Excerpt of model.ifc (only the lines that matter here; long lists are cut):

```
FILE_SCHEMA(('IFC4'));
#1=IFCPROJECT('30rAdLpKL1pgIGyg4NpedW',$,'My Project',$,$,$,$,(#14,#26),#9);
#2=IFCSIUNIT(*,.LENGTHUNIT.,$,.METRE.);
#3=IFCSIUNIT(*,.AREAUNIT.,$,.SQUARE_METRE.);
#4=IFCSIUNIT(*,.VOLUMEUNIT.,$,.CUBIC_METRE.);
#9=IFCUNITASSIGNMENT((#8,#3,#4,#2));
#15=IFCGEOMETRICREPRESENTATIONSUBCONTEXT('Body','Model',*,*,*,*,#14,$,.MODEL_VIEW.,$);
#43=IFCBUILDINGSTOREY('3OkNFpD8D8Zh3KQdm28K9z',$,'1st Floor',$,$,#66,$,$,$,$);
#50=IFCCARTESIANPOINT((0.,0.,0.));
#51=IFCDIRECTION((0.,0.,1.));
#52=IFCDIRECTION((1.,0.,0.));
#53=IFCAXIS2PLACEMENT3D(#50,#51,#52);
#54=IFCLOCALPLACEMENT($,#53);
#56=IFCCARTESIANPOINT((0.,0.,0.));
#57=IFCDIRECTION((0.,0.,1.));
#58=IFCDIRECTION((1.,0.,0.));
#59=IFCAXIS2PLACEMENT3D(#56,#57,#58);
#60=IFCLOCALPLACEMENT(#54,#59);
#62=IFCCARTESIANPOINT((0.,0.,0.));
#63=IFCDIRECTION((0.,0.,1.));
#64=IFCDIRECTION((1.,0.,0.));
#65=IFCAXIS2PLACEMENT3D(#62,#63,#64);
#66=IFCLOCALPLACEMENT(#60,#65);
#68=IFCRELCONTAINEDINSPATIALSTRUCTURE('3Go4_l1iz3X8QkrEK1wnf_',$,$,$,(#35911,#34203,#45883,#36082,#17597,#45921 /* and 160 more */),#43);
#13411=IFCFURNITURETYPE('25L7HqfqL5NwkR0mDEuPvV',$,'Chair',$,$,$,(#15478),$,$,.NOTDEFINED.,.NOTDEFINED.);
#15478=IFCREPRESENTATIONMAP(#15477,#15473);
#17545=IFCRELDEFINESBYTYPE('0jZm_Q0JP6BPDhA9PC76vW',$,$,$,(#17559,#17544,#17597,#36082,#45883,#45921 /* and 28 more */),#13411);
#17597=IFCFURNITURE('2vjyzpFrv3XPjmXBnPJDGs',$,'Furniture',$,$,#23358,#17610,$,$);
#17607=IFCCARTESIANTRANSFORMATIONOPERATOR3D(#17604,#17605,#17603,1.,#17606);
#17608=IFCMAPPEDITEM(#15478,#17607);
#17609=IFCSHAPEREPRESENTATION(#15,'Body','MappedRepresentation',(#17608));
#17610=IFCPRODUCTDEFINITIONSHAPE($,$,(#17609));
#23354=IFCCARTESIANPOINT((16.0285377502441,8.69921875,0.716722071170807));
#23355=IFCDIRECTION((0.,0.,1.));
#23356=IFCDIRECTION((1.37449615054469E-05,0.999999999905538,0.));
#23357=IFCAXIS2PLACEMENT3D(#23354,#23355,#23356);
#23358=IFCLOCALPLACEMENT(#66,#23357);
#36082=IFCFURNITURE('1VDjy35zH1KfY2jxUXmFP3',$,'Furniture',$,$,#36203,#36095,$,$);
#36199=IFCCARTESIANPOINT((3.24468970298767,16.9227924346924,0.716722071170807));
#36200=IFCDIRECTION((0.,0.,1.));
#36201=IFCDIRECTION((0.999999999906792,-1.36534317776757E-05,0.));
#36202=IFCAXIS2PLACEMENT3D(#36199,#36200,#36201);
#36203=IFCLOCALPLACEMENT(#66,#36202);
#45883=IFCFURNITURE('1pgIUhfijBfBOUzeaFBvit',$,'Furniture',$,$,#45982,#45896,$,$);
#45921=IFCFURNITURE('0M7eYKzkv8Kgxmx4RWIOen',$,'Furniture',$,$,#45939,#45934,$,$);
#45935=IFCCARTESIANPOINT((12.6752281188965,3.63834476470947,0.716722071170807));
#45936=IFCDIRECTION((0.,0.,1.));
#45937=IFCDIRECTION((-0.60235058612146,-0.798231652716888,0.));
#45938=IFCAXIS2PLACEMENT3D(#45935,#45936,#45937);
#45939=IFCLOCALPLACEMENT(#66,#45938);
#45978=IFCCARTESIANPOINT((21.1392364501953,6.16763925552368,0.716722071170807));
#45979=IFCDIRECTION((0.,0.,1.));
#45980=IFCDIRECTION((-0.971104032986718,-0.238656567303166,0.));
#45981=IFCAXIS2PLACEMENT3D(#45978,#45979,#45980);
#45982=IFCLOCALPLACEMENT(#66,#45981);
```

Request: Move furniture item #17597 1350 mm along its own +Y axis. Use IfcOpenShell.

```python
import ifcopenshell
import ifcopenshell.api.geometry
import ifcopenshell.util.placement
import ifcopenshell.util.unit

model = ifcopenshell.open("model.ifc")
unit_scale = ifcopenshell.util.unit.calculate_unit_scale(model)

item = model.by_guid("2vjyzpFrv3XPjmXBnPJDGs")
matrix = ifcopenshell.util.placement.get_local_placement(item.ObjectPlacement)
matrix[:3, 3] += matrix[:3, 1] * 1.35 / unit_scale
ifcopenshell.api.geometry.edit_object_placement(model, product=item, matrix=matrix, is_si=False)

print(ifcopenshell.util.placement.get_local_placement(item.ObjectPlacement).round(3) + 0.0)

model.write("model_updated.ifc")
```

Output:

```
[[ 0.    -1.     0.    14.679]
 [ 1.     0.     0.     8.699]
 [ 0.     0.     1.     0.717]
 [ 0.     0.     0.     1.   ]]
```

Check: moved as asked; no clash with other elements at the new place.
